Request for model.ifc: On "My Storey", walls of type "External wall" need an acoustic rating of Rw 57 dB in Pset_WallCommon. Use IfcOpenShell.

First a look at what the model holds.

```python
import ifcopenshell
import ifcopenshell.util.element

model = ifcopenshell.open("model.ifc")
print(model.schema)
storey = next(s for s in model.by_type("IfcBuildingStorey") if s.Name == "My Storey")
walls = [e for e in ifcopenshell.util.element.get_decomposition(storey) if e.is_a("IfcWall")]
seen = {}
for e in walls:
    element_type = ifcopenshell.util.element.get_type(e)
    key = (element_type.Name if element_type != e and element_type else None, ifcopenshell.util.element.get_pset(e, "Pset_WallCommon", "AcousticRating"))
    seen[key] = seen.get(key, 0) + 1
for (name, value), count in sorted(seen.items(), key=str):
    print(count, "x", name, "|", value)
```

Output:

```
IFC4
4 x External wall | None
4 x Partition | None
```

```python
import ifcopenshell
import ifcopenshell.api.pset
import ifcopenshell.util.element

model = ifcopenshell.open("model.ifc")

storey = next(s for s in model.by_type("IfcBuildingStorey") if s.Name == "My Storey")
walls = [e for e in ifcopenshell.util.element.get_decomposition(storey) if e.is_a("IfcWall")]

count = 0
for e in walls:
    element_type = ifcopenshell.util.element.get_type(e)
    if element_type in (None, e) or element_type.Name != "External wall":
        continue
    # add_pset returns the element's existing set when there is one.
    pset = ifcopenshell.api.pset.add_pset(model, product=e, name="Pset_WallCommon")
    ifcopenshell.api.pset.edit_pset(model, pset=pset, properties={"AcousticRating": "Rw 57 dB"})
    count += 1

print(count, "walls updated")

model.write("model_rev.ifc")
```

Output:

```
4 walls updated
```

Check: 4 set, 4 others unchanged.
